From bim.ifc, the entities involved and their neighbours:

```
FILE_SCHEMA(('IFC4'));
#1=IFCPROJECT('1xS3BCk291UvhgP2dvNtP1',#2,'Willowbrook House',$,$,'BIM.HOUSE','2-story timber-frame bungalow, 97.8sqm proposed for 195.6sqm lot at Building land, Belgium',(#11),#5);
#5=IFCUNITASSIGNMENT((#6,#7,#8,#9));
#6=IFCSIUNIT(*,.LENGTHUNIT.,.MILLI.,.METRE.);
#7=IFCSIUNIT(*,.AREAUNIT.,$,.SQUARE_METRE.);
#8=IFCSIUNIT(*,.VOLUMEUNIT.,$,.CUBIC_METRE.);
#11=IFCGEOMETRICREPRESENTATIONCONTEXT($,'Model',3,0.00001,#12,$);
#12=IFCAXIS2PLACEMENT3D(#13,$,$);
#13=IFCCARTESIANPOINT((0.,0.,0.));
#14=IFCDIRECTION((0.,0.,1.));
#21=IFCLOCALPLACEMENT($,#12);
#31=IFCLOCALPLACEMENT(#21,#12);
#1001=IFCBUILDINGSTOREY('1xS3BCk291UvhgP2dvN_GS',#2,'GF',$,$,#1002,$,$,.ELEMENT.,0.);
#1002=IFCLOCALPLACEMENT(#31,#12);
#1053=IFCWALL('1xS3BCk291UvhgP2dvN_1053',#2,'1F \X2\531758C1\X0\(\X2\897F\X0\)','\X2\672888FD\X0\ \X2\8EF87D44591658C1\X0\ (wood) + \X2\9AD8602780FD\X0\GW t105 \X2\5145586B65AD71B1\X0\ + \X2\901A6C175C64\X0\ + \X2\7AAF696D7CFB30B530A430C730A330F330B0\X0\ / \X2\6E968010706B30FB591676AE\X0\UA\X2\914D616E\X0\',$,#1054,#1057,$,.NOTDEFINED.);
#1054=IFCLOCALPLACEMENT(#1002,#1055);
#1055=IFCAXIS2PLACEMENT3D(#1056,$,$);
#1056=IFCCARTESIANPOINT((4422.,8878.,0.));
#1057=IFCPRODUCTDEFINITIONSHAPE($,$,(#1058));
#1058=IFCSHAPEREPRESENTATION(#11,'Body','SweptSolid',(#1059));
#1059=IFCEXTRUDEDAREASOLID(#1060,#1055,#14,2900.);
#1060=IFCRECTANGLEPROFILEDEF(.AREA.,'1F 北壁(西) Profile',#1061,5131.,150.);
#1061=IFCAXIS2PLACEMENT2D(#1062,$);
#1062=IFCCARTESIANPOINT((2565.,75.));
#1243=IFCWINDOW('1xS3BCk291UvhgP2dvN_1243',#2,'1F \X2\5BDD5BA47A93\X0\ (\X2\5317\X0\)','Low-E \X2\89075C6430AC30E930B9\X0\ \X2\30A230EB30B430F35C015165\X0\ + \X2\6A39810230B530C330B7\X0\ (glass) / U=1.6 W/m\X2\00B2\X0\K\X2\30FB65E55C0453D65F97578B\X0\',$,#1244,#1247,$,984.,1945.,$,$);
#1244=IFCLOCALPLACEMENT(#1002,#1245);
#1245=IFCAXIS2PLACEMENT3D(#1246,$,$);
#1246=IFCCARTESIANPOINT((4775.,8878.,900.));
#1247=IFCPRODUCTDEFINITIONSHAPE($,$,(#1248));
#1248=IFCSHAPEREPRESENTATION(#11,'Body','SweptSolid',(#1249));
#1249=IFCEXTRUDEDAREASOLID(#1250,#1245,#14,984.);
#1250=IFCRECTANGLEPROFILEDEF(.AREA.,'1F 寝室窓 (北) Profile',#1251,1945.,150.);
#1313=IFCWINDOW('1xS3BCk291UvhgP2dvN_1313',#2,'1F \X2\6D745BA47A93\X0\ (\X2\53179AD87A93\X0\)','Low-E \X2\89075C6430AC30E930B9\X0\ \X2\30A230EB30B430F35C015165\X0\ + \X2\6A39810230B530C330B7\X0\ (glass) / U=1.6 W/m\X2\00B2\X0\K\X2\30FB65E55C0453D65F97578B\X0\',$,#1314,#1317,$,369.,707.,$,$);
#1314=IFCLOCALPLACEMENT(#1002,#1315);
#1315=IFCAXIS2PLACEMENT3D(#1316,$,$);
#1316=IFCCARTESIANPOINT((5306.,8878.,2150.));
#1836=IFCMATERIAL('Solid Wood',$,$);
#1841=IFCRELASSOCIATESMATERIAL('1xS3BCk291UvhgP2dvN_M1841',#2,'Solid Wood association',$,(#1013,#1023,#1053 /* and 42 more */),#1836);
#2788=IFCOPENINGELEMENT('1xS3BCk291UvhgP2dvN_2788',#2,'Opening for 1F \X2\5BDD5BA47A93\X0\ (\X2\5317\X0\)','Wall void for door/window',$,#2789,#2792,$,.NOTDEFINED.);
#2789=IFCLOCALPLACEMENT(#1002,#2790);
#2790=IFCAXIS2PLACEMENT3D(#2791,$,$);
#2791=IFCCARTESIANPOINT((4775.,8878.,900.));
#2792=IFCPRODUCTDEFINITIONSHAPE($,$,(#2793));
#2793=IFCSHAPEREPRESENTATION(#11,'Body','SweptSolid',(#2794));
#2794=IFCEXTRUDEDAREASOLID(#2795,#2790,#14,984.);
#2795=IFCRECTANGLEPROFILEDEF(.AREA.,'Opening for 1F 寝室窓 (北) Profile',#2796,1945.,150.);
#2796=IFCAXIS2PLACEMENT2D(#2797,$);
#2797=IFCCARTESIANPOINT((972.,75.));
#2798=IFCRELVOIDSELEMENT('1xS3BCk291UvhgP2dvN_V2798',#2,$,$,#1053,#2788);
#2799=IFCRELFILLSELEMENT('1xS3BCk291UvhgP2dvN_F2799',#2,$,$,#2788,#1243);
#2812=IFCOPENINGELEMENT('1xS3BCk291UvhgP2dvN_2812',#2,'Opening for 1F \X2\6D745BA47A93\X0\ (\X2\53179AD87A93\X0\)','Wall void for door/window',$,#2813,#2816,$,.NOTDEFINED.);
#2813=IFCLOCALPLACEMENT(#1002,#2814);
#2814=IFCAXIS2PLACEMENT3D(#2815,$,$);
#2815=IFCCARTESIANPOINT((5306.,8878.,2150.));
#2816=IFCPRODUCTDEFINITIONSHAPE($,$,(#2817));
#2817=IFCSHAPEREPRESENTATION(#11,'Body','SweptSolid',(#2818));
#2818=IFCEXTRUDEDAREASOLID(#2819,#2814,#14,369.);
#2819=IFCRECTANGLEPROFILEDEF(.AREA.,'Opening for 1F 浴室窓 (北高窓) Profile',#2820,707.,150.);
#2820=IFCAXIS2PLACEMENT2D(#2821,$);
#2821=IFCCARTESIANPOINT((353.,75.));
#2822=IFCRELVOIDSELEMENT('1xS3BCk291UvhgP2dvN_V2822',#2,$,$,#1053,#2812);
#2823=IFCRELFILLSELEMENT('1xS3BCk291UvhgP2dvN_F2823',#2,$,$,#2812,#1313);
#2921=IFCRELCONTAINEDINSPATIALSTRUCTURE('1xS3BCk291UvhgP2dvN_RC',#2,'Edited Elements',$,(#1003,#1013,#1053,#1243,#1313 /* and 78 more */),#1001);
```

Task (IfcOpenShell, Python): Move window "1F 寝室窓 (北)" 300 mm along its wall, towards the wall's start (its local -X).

```python
import ifcopenshell
import ifcopenshell.api.geometry
import ifcopenshell.util.placement

model = ifcopenshell.open("bim.ifc")

window = model.by_id(1243)
opening = window.FillsVoids[0].RelatingOpeningElement
wall = opening.VoidsElements[0].RelatingBuildingElement

wall_matrix = ifcopenshell.util.placement.get_local_placement(wall.ObjectPlacement)
shift = wall_matrix[:3, 0] * -300.0
before = ifcopenshell.util.placement.get_local_placement(window.ObjectPlacement)[:3, 3].copy()

# The window is not placed relative to its opening, so move both.
for product in (opening, window):
    matrix = ifcopenshell.util.placement.get_local_placement(product.ObjectPlacement)
    matrix[:3, 3] += shift
    ifcopenshell.api.geometry.edit_object_placement(model, product=product, matrix=matrix, is_si=False)

after = ifcopenshell.util.placement.get_local_placement(window.ObjectPlacement)[:3, 3]
print("window moved by", (after - before).round(3) + 0.0)

model.write("bim_rev.ifc")
```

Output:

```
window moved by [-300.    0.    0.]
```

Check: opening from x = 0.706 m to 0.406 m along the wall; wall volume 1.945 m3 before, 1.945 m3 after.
